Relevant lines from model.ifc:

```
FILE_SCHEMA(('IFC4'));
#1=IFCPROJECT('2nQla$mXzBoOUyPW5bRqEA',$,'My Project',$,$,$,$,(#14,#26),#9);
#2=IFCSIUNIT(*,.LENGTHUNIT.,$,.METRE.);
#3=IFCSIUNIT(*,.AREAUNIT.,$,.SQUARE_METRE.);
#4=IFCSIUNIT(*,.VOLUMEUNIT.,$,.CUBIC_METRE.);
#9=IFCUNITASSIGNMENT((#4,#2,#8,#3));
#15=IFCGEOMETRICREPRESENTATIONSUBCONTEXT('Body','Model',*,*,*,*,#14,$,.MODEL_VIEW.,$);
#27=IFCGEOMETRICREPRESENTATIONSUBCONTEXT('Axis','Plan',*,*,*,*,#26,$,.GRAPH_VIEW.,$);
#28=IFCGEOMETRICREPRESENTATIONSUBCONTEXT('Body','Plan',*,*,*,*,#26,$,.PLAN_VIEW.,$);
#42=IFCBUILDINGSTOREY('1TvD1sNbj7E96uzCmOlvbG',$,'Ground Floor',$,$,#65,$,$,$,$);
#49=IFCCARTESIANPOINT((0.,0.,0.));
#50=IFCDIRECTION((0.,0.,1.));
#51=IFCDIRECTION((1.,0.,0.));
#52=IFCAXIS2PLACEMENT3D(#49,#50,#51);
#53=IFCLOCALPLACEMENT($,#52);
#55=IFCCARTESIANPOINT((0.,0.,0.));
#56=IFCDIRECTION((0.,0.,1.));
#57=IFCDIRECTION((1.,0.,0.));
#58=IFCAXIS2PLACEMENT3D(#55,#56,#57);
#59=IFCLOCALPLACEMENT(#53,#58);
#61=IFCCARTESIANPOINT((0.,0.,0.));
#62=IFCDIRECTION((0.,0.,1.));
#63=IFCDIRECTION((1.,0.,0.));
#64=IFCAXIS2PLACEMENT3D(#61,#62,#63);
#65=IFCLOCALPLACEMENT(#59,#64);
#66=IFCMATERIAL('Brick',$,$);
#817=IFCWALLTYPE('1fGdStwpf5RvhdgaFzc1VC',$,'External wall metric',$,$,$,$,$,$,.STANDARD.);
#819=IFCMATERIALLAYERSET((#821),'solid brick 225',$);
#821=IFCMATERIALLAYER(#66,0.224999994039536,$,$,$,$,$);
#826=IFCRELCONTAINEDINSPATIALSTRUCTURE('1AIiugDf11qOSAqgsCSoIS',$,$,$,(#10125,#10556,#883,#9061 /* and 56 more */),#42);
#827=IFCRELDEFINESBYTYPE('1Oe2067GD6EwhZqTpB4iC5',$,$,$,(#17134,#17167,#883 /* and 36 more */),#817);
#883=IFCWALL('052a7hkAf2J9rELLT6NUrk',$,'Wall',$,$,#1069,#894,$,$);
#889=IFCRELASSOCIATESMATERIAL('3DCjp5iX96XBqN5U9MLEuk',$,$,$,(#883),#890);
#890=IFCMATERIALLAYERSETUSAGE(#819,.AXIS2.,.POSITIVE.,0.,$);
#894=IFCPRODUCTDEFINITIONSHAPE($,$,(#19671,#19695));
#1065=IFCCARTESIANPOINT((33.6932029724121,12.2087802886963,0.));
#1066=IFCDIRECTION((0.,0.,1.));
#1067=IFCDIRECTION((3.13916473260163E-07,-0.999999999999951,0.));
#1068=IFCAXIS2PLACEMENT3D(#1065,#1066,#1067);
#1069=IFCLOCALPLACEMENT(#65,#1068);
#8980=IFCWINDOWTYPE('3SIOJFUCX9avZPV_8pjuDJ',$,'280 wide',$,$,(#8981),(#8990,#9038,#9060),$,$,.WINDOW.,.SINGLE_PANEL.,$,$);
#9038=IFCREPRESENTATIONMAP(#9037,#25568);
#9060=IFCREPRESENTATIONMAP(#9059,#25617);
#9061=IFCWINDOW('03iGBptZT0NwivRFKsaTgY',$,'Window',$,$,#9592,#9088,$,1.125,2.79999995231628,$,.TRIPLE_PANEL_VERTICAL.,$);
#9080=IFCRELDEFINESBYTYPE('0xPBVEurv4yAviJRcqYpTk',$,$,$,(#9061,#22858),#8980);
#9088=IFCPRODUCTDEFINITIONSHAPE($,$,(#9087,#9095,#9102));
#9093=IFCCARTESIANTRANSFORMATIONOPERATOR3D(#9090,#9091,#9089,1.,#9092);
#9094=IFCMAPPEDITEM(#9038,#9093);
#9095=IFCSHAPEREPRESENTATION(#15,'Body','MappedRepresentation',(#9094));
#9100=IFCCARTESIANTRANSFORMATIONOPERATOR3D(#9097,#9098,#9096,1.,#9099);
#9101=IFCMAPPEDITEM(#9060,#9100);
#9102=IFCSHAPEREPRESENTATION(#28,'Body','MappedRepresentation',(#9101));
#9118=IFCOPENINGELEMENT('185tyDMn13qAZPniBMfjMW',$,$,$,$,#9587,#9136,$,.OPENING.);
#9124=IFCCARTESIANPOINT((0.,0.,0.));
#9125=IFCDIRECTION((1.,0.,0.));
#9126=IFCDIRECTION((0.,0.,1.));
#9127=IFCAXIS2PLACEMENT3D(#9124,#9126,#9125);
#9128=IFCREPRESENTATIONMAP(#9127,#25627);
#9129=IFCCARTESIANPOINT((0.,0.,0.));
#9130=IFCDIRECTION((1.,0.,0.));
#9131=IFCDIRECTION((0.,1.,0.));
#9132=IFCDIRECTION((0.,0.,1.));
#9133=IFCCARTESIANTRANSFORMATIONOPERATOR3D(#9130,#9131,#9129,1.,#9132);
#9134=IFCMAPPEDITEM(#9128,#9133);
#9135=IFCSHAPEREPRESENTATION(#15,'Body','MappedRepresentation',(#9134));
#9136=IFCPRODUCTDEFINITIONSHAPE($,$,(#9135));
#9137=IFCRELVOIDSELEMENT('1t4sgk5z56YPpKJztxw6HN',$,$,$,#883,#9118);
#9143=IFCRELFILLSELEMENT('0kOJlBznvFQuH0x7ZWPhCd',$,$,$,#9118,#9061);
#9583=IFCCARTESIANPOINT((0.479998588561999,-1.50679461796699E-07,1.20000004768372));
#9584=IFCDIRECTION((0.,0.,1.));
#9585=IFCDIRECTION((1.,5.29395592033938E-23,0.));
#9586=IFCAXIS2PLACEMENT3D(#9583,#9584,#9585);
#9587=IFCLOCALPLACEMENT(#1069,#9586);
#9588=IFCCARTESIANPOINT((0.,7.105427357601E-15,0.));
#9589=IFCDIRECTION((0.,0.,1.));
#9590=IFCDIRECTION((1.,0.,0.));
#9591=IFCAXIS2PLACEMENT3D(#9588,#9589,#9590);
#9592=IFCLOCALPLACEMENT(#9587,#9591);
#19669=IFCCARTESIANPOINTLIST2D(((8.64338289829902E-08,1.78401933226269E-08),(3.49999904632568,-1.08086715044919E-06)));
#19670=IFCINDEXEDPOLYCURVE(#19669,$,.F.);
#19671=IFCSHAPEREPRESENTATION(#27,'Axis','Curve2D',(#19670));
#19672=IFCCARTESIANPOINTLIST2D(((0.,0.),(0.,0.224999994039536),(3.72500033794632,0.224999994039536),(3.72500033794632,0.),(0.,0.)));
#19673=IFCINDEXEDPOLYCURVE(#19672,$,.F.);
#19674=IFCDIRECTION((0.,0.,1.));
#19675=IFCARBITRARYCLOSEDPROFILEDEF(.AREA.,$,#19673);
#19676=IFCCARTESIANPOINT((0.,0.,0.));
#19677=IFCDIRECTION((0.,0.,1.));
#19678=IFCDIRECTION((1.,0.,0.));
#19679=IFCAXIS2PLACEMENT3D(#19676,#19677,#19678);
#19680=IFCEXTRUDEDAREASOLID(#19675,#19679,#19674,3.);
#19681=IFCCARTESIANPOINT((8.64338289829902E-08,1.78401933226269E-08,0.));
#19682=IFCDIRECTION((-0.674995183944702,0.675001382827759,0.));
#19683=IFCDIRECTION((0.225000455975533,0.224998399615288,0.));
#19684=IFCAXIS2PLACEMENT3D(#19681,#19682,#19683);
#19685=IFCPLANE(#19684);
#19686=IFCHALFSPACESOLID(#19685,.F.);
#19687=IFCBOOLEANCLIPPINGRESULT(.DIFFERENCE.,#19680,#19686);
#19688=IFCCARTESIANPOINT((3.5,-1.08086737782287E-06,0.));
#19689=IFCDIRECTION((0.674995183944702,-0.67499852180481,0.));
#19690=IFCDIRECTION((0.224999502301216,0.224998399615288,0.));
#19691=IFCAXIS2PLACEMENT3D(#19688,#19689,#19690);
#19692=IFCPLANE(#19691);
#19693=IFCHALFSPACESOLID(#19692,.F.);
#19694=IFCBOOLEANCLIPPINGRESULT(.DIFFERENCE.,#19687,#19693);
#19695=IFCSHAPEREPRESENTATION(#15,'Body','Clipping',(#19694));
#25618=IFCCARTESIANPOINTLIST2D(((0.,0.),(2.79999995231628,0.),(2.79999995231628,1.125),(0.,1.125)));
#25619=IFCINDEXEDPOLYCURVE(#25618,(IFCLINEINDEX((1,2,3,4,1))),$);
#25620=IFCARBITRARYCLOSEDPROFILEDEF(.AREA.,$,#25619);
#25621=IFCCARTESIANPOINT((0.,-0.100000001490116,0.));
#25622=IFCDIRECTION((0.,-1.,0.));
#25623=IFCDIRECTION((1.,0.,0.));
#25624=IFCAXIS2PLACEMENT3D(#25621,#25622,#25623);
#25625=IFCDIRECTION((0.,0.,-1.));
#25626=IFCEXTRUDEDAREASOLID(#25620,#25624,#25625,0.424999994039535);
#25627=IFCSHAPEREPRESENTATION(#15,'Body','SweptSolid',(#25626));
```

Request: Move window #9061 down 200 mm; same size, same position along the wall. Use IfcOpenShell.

```python
import numpy as np
import ifcopenshell
import ifcopenshell.api.geometry
import ifcopenshell.util.placement
import ifcopenshell.util.unit

model = ifcopenshell.open("model.ifc")
unit_scale = ifcopenshell.util.unit.calculate_unit_scale(model)

window = model.by_id(9061)
opening = window.FillsVoids[0].RelatingOpeningElement
dz = -0.2

shift = np.array([0.0, 0.0, dz])
# The window is placed relative to its opening, so it follows when the opening moves.
matrix = ifcopenshell.util.placement.get_local_placement(opening.ObjectPlacement)
matrix[:3, 3] += shift
ifcopenshell.api.geometry.edit_object_placement(
    model, product=opening, matrix=matrix, is_si=False, should_transform_children=True
)

print(f"moved by {dz * unit_scale:+.3f} m")

model.write("model_edited.ifc")
```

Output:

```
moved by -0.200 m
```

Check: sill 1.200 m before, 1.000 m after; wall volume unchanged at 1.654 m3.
